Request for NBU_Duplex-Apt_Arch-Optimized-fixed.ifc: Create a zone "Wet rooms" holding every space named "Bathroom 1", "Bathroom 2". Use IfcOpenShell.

First a look at what the model holds.

```python
import ifcopenshell

model = ifcopenshell.open("NBU_Duplex-Apt_Arch-Optimized-fixed.ifc")
print(model.schema)
seen = {}
for space in model.by_type("IfcSpace"):
    seen[space.LongName] = seen.get(space.LongName, 0) + 1
for name, count in sorted(seen.items(), key=str):
    print(count, "x", name)
print("zones:", [z.Name for z in model.by_type("IfcZone")][:20])
```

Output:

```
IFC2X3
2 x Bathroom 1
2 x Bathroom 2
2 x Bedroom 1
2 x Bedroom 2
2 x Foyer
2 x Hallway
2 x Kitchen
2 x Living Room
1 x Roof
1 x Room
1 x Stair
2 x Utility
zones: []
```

```python
import ifcopenshell
import ifcopenshell.api.group
import ifcopenshell.api.root

model = ifcopenshell.open("NBU_Duplex-Apt_Arch-Optimized-fixed.ifc")

names = {"Bathroom 1", "Bathroom 2"}
spaces = [s for s in model.by_type("IfcSpace") if s.LongName in names]

zone = ifcopenshell.api.root.create_entity(model, ifc_class="IfcZone", name="Wet rooms")
ifcopenshell.api.group.assign_group(model, products=spaces, group=zone)
print(len(spaces), "spaces in", zone.Name)

model.write("NBU_Duplex-Apt_Arch-Optimized-fixed_v2.ifc")
```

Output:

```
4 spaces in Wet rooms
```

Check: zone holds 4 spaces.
